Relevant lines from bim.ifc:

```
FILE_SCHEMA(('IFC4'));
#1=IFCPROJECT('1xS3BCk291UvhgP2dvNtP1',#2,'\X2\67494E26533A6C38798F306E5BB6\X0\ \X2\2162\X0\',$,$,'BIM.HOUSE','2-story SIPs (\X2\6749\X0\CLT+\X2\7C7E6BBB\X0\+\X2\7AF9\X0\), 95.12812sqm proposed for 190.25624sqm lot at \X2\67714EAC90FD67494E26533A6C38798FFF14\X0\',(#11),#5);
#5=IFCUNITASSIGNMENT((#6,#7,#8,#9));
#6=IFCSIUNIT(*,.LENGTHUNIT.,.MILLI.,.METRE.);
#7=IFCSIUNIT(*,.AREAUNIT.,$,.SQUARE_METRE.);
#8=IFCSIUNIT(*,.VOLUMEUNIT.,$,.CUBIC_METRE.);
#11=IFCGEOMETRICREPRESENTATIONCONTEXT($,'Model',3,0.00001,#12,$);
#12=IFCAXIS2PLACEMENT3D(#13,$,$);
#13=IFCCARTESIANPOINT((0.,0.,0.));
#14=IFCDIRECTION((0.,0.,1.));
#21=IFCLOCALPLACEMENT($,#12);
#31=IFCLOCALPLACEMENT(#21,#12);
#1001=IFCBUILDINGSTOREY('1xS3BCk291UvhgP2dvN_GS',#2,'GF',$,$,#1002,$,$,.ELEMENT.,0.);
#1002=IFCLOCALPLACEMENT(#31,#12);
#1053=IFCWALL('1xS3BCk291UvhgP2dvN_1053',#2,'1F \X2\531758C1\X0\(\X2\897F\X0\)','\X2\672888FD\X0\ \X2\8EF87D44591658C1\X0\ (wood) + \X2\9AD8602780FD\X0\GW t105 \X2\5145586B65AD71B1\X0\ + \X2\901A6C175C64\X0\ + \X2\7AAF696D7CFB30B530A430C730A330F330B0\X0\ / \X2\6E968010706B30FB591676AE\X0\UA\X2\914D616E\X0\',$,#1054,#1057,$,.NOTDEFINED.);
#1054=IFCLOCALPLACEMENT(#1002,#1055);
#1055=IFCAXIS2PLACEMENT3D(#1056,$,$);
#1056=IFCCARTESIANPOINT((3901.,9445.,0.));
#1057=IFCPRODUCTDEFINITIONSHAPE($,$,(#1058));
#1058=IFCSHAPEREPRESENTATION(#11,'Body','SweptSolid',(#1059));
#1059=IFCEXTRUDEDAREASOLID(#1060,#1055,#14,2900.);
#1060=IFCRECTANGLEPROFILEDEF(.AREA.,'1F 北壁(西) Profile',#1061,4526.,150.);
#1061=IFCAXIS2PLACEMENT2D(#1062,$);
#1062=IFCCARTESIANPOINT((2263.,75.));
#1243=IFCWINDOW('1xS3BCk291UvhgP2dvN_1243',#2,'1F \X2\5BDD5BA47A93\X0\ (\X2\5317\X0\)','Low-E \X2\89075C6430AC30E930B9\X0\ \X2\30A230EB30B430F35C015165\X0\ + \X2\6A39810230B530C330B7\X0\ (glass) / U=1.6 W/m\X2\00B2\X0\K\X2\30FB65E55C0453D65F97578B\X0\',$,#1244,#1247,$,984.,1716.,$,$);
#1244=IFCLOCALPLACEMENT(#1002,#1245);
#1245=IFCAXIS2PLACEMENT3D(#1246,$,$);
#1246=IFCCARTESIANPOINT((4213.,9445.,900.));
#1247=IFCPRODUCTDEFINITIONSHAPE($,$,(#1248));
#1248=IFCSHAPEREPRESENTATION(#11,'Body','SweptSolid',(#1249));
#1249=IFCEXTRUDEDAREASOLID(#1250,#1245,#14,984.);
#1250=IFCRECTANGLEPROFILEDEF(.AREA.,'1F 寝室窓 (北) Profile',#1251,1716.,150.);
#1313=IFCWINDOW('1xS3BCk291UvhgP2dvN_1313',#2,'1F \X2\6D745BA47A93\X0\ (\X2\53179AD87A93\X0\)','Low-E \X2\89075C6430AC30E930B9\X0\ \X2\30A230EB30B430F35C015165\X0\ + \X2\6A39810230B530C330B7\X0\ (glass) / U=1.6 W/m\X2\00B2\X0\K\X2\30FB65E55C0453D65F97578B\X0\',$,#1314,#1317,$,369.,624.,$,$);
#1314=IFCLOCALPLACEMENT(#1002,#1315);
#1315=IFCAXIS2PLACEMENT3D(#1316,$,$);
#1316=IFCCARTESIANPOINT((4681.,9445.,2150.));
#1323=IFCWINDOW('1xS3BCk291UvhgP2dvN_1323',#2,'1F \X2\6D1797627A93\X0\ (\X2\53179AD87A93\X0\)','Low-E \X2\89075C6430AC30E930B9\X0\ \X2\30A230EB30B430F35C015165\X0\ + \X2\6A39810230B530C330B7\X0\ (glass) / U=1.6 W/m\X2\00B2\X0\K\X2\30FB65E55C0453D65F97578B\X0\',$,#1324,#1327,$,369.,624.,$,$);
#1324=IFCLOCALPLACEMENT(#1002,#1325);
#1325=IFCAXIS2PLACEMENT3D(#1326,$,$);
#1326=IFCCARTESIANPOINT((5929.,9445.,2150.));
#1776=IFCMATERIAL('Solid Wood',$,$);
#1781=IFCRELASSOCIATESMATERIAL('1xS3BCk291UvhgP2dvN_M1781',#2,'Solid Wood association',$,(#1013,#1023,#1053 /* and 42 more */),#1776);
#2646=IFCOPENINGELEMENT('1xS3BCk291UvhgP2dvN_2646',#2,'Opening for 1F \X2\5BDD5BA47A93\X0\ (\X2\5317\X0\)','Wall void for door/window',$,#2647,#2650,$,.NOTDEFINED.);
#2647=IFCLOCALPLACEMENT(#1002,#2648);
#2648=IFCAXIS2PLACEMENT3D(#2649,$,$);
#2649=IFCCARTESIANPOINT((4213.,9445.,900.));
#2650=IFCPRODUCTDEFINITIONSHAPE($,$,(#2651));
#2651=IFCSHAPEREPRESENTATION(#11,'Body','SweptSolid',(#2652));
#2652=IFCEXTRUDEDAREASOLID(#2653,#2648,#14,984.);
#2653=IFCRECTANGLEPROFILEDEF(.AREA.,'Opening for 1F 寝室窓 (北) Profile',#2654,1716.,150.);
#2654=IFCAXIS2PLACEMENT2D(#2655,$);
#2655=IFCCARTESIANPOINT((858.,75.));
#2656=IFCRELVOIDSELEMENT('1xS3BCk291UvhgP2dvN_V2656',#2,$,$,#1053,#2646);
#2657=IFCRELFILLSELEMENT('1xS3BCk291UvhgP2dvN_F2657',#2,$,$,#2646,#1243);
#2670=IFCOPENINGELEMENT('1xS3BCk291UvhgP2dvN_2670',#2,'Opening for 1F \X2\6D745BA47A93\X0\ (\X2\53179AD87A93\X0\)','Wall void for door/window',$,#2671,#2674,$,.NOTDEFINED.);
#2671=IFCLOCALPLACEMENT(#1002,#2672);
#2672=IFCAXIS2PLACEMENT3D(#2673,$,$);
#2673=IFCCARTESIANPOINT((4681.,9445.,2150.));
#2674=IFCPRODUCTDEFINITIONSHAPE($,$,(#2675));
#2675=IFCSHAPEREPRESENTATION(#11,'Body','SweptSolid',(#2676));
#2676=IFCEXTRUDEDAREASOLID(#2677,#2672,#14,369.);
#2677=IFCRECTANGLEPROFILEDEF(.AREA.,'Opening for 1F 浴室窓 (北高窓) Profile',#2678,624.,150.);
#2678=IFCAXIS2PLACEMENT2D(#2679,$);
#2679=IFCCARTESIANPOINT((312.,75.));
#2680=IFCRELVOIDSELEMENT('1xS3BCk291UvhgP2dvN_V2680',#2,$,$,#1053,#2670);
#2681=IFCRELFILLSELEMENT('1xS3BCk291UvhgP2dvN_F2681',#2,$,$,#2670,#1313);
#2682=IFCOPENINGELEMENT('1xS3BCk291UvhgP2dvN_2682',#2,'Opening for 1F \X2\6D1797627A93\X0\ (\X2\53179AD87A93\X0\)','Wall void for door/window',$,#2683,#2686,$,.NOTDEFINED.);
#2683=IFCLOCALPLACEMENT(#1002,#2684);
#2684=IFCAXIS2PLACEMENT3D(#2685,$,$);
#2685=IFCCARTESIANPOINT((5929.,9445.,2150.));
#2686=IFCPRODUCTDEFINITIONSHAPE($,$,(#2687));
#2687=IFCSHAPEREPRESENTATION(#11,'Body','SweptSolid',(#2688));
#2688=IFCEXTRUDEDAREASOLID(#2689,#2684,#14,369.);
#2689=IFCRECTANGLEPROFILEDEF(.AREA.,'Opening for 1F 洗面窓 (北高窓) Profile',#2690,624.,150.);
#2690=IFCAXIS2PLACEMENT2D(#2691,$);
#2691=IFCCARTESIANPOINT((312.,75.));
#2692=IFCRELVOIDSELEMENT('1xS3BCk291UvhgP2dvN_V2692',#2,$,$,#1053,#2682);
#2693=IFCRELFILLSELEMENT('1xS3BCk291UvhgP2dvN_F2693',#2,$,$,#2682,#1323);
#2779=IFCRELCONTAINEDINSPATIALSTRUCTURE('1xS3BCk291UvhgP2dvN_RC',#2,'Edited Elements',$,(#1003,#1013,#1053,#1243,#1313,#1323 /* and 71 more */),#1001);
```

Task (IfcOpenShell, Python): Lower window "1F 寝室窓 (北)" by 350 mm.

```python
import numpy as np
import ifcopenshell
import ifcopenshell.api.geometry
import ifcopenshell.util.placement
import ifcopenshell.util.unit

model = ifcopenshell.open("bim.ifc")
unit_scale = ifcopenshell.util.unit.calculate_unit_scale(model)

window = model.by_guid("1xS3BCk291UvhgP2dvN_1243")
opening = window.FillsVoids[0].RelatingOpeningElement
dz = -350.0

shift = np.array([0.0, 0.0, dz])
# The window is not placed relative to its opening, so move both.
for product in (opening, window):
    matrix = ifcopenshell.util.placement.get_local_placement(product.ObjectPlacement)
    matrix[:3, 3] += shift
    ifcopenshell.api.geometry.edit_object_placement(model, product=product, matrix=matrix, is_si=False)

print(f"moved by {dz * unit_scale:+.3f} m")

model.write("bim_edited.ifc")
```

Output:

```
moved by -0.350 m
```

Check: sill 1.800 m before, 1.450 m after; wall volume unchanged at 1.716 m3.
